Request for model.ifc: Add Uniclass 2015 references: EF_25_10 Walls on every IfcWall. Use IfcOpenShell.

First a look at what the model holds.

```python
import ifcopenshell

model = ifcopenshell.open("model.ifc")
print(model.schema)
print("classifications:", [c.Name for c in model.by_type("IfcClassification")])
for ifc_class in ("IfcDoor", "IfcRoof", "IfcStair", "IfcWall", "IfcWindow"):
    print(ifc_class, len(model.by_type(ifc_class)))
```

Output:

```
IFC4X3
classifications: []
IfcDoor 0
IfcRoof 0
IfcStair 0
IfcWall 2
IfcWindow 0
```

```python
import ifcopenshell
import ifcopenshell.api.classification

model = ifcopenshell.open("model.ifc")

system = ifcopenshell.api.classification.add_classification(model, classification="Uniclass 2015")

codes = {
    "IfcWall": ("EF_25_10", "Walls"),
}
for ifc_class, (code, name) in codes.items():
    products = model.by_type(ifc_class)
    ifcopenshell.api.classification.add_reference(
        model, products=products, classification=system, identification=code, name=name
    )
    print(code, len(products))

model.write("model_v2.ifc")
```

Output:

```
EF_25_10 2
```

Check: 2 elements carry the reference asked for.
